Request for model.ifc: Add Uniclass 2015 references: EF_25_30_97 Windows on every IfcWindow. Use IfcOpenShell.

First a look at what the model holds.

```python
import ifcopenshell

model = ifcopenshell.open("model.ifc")
print(model.schema)
print("classifications:", [c.Name for c in model.by_type("IfcClassification")])
for ifc_class in ("IfcDoor", "IfcRoof", "IfcStair", "IfcWall", "IfcWindow"):
    print(ifc_class, len(model.by_type(ifc_class)))
```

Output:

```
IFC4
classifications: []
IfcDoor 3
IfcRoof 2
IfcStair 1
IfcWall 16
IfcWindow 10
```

```python
import ifcopenshell
import ifcopenshell.api.classification

model = ifcopenshell.open("model.ifc")

system = ifcopenshell.api.classification.add_classification(model, classification="Uniclass 2015")

codes = {
    "IfcWindow": ("EF_25_30_97", "Windows"),
}
for ifc_class, (code, name) in codes.items():
    products = model.by_type(ifc_class)
    ifcopenshell.api.classification.add_reference(
        model, products=products, classification=system, identification=code, name=name
    )
    print(code, len(products))

model.write("model_edited.ifc")
```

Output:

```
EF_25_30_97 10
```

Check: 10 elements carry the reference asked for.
